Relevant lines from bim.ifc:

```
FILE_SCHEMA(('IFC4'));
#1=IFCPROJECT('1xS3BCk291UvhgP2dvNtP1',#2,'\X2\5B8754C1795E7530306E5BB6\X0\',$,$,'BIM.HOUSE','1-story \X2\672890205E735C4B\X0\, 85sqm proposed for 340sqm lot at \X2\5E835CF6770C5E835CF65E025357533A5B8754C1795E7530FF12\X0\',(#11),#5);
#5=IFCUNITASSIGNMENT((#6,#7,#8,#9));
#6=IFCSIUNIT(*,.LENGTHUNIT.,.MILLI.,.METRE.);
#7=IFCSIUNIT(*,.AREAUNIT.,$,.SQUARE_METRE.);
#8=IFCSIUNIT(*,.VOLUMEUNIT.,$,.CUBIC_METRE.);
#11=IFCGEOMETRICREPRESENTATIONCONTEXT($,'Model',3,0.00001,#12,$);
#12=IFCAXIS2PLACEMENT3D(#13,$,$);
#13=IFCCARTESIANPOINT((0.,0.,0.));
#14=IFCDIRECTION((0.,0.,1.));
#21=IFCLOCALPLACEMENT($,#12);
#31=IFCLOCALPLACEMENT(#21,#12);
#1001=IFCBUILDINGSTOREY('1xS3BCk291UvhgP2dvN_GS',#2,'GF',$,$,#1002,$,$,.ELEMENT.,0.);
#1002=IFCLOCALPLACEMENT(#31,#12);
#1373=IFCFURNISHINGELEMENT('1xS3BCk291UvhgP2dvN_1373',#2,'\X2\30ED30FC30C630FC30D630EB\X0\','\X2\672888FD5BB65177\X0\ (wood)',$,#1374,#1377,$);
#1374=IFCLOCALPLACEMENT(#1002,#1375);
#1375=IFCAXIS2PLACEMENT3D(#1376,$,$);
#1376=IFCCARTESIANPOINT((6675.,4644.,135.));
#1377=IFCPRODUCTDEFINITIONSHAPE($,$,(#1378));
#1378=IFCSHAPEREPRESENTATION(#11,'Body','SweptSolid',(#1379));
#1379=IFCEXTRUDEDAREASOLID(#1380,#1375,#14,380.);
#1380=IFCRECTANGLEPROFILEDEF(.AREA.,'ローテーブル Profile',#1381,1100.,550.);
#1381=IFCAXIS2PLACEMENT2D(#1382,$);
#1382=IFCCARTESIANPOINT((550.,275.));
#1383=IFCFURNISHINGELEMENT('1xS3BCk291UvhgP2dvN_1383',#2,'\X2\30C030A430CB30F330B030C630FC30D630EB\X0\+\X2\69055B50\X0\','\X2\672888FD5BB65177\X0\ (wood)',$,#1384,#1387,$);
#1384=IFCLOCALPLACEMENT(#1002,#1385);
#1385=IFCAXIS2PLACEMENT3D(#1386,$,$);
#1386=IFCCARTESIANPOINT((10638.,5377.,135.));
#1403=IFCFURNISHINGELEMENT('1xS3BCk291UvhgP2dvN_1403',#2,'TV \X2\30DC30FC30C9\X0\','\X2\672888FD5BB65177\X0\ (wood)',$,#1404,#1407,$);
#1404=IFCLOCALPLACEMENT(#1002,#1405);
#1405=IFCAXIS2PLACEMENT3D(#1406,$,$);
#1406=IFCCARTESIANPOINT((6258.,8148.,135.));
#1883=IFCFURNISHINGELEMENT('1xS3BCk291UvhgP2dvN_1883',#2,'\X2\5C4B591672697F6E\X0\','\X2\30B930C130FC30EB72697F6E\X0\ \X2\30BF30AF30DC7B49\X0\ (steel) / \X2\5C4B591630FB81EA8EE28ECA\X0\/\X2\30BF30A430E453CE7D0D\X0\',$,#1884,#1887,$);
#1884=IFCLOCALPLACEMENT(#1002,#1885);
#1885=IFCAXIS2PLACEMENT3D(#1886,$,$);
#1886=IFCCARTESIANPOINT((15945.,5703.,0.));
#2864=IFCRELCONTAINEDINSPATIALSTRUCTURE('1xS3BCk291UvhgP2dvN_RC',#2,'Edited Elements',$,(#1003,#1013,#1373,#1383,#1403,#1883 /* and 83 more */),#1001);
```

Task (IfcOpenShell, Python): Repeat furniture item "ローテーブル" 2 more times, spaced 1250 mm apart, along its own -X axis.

```python
import ifcopenshell
import ifcopenshell.api.geometry
import ifcopenshell.api.root
import ifcopenshell.util.element
import ifcopenshell.util.placement
import ifcopenshell.util.unit

model = ifcopenshell.open("bim.ifc")
unit_scale = ifcopenshell.util.unit.calculate_unit_scale(model)


def reuse_history(source, copy):
    """copy_class also copies each property set's owner history, people and application; keep the originals."""
    for rel in copy.IsDefinedBy:
        if rel.is_a("IfcRelDefinesByProperties") and (history := rel.RelatingPropertyDefinition.OwnerHistory):
            rel.RelatingPropertyDefinition.OwnerHistory = source.OwnerHistory
            ifcopenshell.util.element.remove_deep2(model, history)


source = model.by_id(1373)
base = ifcopenshell.util.placement.get_local_placement(source.ObjectPlacement)
step = -base[:3, 0] * 1.25 / unit_scale

for i in range(1, 3):
    copy = ifcopenshell.api.root.copy_class(model, product=source)
    copy.Representation = ifcopenshell.util.element.copy_deep(
        model, source.Representation, exclude=["IfcGeometricRepresentationContext", "IfcRepresentationMap"]
    )
    reuse_history(source, copy)
    matrix = base.copy()
    matrix[:3, 3] += i * step
    print("added at", matrix[:3, 3].round(3) + 0.0)
    ifcopenshell.api.geometry.edit_object_placement(model, product=copy, matrix=matrix, is_si=False)

model.write("bim_v2.ifc")
```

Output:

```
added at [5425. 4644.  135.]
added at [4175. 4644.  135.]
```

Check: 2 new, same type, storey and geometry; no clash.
